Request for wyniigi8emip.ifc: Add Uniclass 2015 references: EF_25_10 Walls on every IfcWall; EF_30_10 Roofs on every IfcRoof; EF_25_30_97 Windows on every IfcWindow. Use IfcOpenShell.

First a look at what the model holds.

```python
import ifcopenshell

model = ifcopenshell.open("wyniigi8emip.ifc")
print(model.schema)
print("classifications:", [c.Name for c in model.by_type("IfcClassification")])
for ifc_class in ("IfcDoor", "IfcRoof", "IfcStair", "IfcWall", "IfcWindow"):
    print(ifc_class, len(model.by_type(ifc_class)))
```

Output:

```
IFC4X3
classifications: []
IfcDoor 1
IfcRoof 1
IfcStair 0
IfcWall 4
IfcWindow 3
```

```python
import ifcopenshell
import ifcopenshell.api.classification

model = ifcopenshell.open("wyniigi8emip.ifc")

system = ifcopenshell.api.classification.add_classification(model, classification="Uniclass 2015")

codes = {
    "IfcWall": ("EF_25_10", "Walls"),
    "IfcRoof": ("EF_30_10", "Roofs"),
    "IfcWindow": ("EF_25_30_97", "Windows"),
}
for ifc_class, (code, name) in codes.items():
    products = model.by_type(ifc_class)
    ifcopenshell.api.classification.add_reference(
        model, products=products, classification=system, identification=code, name=name
    )
    print(code, len(products))

model.write("wyniigi8emip-out.ifc")
```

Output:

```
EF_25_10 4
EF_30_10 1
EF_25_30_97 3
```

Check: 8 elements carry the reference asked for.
